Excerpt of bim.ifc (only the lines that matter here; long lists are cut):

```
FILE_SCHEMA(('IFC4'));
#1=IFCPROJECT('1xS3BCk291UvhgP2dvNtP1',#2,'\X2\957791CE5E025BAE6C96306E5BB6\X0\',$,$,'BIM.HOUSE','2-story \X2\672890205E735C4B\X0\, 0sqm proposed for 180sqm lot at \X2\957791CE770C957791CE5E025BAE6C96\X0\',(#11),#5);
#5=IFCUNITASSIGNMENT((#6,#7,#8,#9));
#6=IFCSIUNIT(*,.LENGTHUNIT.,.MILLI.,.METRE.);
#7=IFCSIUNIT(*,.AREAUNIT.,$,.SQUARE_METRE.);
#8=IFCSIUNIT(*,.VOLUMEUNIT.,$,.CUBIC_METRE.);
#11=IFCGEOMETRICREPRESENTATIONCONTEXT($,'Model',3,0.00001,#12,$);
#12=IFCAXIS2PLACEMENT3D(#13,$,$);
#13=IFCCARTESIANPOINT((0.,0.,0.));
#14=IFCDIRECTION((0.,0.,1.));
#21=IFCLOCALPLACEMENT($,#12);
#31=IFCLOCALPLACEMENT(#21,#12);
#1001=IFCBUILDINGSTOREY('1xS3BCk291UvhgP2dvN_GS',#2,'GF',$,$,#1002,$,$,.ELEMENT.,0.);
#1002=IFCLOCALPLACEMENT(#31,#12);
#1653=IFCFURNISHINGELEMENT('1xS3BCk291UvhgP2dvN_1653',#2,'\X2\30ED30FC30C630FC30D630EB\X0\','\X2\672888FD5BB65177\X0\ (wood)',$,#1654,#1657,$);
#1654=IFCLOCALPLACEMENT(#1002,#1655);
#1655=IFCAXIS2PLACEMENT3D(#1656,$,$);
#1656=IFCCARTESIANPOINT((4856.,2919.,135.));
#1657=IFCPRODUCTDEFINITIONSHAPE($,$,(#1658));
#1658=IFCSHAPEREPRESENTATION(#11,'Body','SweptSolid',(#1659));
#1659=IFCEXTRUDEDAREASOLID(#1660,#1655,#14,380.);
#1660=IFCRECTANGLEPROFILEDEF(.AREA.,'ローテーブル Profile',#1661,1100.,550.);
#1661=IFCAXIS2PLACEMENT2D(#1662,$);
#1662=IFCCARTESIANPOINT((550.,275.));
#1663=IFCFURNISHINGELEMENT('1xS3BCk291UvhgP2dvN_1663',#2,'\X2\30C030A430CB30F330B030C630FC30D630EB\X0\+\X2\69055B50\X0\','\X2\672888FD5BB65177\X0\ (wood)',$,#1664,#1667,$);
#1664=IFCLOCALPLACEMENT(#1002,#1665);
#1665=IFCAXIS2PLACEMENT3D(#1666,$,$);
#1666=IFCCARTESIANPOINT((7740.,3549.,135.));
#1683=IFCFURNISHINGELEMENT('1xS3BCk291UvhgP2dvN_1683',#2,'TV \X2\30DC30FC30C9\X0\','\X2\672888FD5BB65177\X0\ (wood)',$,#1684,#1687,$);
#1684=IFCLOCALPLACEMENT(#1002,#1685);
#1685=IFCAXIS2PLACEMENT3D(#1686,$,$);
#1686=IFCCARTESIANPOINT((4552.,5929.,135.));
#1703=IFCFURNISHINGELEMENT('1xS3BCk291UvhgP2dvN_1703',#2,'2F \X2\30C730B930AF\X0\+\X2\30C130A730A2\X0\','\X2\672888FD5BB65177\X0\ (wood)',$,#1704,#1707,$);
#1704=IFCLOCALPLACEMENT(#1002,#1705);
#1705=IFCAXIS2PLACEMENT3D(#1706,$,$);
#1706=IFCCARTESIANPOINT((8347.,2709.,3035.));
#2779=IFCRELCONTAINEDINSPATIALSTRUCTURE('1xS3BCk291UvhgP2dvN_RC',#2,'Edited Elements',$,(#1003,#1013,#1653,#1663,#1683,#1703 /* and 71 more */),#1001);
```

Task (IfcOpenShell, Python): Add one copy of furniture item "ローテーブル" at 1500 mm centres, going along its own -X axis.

```python
import ifcopenshell
import ifcopenshell.api.geometry
import ifcopenshell.api.root
import ifcopenshell.util.element
import ifcopenshell.util.placement

model = ifcopenshell.open("bim.ifc")


def reuse_history(source, copy):
    """copy_class also copies each property set's owner history, people and application; keep the originals."""
    for rel in copy.IsDefinedBy:
        if rel.is_a("IfcRelDefinesByProperties") and (history := rel.RelatingPropertyDefinition.OwnerHistory):
            rel.RelatingPropertyDefinition.OwnerHistory = source.OwnerHistory
            ifcopenshell.util.element.remove_deep2(model, history)


source = model.by_guid("1xS3BCk291UvhgP2dvN_1653")
base = ifcopenshell.util.placement.get_local_placement(source.ObjectPlacement)
step = -base[:3, 0] * 1500.0

for i in range(1, 2):
    copy = ifcopenshell.api.root.copy_class(model, product=source)
    copy.Representation = ifcopenshell.util.element.copy_deep(
        model, source.Representation, exclude=["IfcGeometricRepresentationContext", "IfcRepresentationMap"]
    )
    reuse_history(source, copy)
    matrix = base.copy()
    matrix[:3, 3] += i * step
    print("added at", matrix[:3, 3].round(3) + 0.0)
    ifcopenshell.api.geometry.edit_object_placement(model, product=copy, matrix=matrix, is_si=False)

model.write("bim_edited.ifc")
```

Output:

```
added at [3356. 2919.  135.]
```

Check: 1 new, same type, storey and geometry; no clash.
